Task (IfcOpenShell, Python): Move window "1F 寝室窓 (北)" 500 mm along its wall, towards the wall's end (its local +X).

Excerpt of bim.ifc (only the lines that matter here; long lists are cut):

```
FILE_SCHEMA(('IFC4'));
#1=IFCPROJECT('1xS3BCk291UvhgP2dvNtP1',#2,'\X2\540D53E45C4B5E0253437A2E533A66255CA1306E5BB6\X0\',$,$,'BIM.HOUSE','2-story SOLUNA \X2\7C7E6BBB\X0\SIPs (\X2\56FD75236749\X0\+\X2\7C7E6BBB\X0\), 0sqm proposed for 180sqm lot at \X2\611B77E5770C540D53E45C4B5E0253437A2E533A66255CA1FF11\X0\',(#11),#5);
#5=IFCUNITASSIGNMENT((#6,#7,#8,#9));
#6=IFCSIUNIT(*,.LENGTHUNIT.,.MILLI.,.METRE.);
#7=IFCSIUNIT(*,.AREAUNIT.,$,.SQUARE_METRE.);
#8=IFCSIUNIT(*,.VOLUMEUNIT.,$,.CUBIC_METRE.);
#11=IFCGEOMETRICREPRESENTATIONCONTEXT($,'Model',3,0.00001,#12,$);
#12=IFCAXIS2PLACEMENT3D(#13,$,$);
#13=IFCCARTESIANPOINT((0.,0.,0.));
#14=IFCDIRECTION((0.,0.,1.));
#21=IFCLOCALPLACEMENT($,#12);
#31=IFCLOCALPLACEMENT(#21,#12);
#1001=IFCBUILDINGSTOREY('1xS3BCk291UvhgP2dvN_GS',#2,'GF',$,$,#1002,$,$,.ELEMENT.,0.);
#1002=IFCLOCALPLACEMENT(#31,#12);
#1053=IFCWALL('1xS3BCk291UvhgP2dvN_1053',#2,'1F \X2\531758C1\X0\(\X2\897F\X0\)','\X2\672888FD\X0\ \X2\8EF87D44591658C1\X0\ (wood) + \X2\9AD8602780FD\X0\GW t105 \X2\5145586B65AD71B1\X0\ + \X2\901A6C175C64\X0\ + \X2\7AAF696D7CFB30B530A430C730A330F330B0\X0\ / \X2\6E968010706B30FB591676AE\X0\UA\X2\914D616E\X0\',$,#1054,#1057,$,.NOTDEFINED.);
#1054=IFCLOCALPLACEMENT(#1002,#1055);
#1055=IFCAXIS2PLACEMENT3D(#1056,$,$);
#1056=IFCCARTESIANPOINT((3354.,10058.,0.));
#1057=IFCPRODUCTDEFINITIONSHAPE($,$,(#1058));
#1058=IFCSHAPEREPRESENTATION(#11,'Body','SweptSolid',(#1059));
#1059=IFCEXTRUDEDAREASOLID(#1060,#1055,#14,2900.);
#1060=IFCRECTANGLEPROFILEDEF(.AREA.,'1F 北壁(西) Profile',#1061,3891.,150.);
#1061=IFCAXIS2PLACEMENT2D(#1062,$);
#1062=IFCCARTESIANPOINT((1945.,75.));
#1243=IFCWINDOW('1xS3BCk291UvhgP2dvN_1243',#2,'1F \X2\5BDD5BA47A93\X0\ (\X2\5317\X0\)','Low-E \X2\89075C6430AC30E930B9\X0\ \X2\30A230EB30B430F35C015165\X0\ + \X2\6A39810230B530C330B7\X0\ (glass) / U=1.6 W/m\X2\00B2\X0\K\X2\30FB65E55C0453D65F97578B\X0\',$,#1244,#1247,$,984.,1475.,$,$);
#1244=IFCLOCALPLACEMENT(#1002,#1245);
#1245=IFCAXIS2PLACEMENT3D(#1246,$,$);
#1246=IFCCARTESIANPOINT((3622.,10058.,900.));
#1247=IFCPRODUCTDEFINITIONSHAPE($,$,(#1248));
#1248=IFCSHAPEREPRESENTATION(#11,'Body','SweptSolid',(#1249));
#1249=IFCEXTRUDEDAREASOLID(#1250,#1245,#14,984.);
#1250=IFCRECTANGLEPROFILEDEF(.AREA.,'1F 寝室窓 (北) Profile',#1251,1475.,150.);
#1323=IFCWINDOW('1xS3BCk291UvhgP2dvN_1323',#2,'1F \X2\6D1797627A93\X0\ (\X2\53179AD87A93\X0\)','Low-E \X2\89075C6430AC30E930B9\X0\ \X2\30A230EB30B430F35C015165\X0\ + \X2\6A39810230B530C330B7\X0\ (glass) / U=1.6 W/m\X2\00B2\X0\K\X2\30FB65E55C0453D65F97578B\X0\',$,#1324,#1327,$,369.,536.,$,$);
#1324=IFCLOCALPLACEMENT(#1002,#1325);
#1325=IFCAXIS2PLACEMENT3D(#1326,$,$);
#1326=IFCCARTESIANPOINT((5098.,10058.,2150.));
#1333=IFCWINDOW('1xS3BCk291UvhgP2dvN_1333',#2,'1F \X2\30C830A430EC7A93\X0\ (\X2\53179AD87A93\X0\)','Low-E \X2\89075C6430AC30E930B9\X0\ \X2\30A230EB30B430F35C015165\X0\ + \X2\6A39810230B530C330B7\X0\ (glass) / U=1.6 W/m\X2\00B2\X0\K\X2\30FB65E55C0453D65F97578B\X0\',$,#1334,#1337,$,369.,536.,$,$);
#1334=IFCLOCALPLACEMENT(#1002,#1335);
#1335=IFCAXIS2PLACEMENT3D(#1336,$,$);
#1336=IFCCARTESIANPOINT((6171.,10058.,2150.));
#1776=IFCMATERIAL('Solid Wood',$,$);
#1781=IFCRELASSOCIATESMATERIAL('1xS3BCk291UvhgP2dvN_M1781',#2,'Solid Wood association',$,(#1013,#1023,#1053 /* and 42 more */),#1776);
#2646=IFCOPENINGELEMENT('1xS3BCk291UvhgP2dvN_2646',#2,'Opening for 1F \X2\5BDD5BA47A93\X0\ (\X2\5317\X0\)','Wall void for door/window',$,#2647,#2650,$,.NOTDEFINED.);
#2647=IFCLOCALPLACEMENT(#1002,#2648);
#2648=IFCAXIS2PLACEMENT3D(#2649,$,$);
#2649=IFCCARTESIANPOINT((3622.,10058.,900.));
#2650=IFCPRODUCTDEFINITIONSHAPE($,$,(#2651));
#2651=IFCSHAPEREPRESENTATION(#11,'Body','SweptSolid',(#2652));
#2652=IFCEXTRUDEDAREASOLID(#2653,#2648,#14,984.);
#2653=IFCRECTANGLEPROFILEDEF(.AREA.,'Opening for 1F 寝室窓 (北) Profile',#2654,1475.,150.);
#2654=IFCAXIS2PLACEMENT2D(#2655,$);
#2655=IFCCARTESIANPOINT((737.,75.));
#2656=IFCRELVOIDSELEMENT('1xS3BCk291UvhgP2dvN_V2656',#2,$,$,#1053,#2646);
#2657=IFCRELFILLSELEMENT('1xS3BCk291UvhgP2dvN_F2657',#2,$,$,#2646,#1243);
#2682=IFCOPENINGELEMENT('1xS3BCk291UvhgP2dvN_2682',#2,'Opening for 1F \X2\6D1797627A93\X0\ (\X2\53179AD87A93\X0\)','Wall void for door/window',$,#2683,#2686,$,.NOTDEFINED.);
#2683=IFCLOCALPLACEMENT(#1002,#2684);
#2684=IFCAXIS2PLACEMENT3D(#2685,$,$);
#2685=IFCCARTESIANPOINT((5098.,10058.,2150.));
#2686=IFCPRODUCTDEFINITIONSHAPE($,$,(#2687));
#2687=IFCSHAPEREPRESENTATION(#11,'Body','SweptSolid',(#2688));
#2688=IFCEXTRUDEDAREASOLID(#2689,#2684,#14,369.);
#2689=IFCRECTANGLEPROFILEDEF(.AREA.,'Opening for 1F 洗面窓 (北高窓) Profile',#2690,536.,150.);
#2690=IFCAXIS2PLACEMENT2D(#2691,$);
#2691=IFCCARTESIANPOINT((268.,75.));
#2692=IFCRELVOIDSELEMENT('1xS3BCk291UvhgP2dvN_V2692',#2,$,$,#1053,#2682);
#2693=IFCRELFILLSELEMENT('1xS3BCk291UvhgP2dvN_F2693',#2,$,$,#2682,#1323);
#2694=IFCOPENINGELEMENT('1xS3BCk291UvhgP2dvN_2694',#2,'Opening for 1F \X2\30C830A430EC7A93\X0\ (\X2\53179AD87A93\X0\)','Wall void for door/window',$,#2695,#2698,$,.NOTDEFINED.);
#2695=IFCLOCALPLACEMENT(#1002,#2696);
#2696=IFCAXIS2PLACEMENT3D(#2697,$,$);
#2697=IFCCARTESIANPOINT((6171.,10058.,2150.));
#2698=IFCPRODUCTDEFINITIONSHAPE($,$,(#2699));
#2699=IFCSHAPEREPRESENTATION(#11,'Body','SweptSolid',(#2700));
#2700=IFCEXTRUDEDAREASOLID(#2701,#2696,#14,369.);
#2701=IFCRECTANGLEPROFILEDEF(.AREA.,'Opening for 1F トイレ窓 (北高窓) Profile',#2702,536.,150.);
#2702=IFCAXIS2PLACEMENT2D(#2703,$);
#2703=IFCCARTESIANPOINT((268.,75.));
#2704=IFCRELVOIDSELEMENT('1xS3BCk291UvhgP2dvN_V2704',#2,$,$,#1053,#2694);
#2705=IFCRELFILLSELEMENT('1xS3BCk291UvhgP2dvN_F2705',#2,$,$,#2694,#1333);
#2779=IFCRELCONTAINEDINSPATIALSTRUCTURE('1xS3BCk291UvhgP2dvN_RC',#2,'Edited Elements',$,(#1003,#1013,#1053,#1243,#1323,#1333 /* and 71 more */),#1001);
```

```python
import ifcopenshell
import ifcopenshell.api.geometry
import ifcopenshell.util.placement
import ifcopenshell.util.unit

model = ifcopenshell.open("bim.ifc")
unit_scale = ifcopenshell.util.unit.calculate_unit_scale(model)

window = model.by_guid("1xS3BCk291UvhgP2dvN_1243")
opening = window.FillsVoids[0].RelatingOpeningElement
wall = opening.VoidsElements[0].RelatingBuildingElement

wall_matrix = ifcopenshell.util.placement.get_local_placement(wall.ObjectPlacement)
shift = wall_matrix[:3, 0] * 0.5 / unit_scale
before = ifcopenshell.util.placement.get_local_placement(window.ObjectPlacement)[:3, 3].copy()

# The window is not placed relative to its opening, so move both.
for product in (opening, window):
    matrix = ifcopenshell.util.placement.get_local_placement(product.ObjectPlacement)
    matrix[:3, 3] += shift
    ifcopenshell.api.geometry.edit_object_placement(model, product=product, matrix=matrix, is_si=False)

after = ifcopenshell.util.placement.get_local_placement(window.ObjectPlacement)[:3, 3]
print("window moved by", (after - before).round(3) + 0.0)

model.write("bim_v2.ifc")
```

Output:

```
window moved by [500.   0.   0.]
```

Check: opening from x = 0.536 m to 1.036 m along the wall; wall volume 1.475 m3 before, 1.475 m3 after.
